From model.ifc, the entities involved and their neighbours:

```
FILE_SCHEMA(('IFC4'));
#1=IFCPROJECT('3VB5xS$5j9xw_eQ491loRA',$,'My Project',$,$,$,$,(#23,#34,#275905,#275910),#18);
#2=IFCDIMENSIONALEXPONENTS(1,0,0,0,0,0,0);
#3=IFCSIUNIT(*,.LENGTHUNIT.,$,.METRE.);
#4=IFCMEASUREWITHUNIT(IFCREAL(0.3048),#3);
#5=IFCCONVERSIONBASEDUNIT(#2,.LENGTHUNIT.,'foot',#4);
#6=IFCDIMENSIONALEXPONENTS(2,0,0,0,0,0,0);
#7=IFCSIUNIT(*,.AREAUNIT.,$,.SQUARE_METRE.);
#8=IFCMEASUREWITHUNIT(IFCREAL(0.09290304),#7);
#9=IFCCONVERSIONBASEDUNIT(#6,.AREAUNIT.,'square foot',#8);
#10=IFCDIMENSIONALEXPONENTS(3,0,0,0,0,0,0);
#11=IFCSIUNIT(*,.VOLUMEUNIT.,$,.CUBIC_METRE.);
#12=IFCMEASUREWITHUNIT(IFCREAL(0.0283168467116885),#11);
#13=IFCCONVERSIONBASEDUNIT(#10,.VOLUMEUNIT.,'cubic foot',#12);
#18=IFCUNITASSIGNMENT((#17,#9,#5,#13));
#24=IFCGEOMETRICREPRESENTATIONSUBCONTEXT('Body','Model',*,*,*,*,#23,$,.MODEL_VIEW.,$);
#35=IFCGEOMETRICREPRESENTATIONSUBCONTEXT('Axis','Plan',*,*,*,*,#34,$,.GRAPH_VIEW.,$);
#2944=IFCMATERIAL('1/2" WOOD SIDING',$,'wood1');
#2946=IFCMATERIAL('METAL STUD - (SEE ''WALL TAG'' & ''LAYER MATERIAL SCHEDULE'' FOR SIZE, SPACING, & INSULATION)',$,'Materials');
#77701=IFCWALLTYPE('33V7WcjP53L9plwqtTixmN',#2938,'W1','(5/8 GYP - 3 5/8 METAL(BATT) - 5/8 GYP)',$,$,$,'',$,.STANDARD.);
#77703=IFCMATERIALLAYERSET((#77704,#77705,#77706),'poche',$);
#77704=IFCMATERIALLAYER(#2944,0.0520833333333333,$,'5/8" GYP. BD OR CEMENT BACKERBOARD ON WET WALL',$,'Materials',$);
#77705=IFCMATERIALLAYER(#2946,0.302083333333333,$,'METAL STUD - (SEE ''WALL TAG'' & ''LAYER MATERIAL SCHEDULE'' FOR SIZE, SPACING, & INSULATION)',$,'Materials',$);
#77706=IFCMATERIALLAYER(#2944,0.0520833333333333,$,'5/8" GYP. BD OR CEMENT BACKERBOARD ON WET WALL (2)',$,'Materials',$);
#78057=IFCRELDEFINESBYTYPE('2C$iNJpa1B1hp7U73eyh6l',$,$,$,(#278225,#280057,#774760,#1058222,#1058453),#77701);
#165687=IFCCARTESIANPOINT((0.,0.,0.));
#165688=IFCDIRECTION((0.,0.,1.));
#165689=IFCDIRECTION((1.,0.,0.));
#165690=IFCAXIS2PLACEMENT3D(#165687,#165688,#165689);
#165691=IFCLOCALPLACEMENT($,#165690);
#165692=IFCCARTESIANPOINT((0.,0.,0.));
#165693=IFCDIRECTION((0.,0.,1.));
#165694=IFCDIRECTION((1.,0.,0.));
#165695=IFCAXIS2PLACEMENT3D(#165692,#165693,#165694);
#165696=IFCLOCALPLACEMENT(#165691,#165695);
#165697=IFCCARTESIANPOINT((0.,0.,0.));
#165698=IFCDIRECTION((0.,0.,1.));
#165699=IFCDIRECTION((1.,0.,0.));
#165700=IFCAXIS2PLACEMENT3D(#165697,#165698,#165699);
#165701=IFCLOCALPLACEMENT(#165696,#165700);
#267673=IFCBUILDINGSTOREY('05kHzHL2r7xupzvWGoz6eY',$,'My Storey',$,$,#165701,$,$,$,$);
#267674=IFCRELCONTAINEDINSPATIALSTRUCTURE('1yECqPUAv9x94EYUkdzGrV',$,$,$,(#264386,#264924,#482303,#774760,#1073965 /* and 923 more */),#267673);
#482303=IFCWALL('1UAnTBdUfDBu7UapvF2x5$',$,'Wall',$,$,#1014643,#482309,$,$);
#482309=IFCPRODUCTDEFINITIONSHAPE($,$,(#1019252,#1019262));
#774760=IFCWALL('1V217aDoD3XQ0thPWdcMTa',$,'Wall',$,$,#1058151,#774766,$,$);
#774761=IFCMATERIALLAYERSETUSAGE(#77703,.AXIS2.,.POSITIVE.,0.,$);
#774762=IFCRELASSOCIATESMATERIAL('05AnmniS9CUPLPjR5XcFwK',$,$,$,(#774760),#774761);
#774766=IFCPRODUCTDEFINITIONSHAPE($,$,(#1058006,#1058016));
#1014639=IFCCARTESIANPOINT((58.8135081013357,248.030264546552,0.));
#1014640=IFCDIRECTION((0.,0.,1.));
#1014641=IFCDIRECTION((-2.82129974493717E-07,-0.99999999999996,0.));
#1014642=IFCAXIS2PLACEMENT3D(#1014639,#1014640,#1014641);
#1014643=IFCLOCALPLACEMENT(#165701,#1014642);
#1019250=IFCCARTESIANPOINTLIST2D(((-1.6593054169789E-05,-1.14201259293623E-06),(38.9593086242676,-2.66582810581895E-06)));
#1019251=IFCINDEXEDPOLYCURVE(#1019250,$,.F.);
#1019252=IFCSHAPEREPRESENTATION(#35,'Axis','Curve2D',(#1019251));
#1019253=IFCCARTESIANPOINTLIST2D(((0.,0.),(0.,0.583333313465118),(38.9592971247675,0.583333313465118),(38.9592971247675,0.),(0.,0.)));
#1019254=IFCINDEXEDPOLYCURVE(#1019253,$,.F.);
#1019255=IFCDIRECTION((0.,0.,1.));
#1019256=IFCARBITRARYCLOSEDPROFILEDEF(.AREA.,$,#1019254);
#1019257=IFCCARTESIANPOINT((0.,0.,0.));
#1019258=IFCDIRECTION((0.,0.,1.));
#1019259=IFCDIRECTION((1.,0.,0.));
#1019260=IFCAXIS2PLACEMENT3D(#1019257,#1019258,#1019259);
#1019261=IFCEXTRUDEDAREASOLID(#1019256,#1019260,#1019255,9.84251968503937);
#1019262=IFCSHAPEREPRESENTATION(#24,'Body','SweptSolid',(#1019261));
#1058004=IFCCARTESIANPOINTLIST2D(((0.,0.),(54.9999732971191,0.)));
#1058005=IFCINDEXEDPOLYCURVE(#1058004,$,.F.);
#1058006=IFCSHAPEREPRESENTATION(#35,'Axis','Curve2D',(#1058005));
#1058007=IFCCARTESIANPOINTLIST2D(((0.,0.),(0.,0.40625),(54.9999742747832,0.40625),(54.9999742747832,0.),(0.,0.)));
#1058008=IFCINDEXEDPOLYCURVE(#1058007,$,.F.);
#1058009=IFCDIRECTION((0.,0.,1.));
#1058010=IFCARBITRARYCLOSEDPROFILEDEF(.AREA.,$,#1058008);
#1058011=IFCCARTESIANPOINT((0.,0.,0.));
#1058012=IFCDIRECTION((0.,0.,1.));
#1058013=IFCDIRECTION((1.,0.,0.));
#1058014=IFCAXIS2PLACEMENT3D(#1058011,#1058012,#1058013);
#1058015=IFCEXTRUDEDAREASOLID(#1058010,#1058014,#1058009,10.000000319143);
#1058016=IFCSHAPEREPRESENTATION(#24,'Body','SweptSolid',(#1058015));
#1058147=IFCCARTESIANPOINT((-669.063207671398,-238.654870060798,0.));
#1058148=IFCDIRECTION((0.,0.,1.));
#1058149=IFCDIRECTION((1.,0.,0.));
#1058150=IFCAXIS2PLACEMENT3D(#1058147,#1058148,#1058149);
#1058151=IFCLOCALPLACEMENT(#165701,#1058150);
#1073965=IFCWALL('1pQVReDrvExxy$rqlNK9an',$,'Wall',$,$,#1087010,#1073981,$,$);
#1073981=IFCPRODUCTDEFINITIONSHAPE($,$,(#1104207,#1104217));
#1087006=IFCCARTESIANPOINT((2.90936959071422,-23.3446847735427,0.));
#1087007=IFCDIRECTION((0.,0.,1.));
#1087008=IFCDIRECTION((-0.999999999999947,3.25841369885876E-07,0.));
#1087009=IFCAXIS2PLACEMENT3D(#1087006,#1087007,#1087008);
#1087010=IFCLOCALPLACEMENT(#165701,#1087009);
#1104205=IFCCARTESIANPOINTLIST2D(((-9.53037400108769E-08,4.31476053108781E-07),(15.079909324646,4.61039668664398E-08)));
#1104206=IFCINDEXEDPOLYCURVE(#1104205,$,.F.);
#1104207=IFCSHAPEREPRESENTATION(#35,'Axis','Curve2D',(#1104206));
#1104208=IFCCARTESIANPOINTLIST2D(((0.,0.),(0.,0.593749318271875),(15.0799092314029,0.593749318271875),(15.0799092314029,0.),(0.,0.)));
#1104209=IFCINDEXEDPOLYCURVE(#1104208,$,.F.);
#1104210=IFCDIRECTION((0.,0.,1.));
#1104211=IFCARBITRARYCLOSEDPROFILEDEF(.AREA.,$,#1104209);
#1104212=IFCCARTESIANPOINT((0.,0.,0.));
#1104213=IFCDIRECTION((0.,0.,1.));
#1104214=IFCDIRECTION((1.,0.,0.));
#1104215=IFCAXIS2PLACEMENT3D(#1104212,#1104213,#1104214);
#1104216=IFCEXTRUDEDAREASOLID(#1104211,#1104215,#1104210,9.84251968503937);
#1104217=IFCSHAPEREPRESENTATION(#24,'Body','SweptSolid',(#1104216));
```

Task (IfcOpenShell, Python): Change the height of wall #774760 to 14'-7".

```python
import ifcopenshell
import ifcopenshell.geom
import ifcopenshell.util.representation
import ifcopenshell.util.shape
import ifcopenshell.util.unit

model = ifcopenshell.open("model.ifc")
unit_scale = ifcopenshell.util.unit.calculate_unit_scale(model)
settings = ifcopenshell.geom.settings()


def volume(element):
    """Net volume in cubic metres, openings subtracted."""
    shape = ifcopenshell.geom.create_shape(settings, element)
    return ifcopenshell.util.shape.get_volume(shape.geometry)


wall = model.by_id(774760)
before = volume(wall)

body = ifcopenshell.util.representation.get_representation(wall, "Model", "Body")
solid = body.Items[0]
old_height = solid.Depth
solid.Depth = 175 * 0.0254 / unit_scale
after = volume(wall)

print(f"height {old_height:g} -> {solid.Depth:g}, volume {before:.3f} -> {after:.3f} m3")

model.write("model-out.ifc")
```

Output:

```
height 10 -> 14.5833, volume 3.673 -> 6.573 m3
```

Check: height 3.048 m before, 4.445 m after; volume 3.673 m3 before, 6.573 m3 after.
